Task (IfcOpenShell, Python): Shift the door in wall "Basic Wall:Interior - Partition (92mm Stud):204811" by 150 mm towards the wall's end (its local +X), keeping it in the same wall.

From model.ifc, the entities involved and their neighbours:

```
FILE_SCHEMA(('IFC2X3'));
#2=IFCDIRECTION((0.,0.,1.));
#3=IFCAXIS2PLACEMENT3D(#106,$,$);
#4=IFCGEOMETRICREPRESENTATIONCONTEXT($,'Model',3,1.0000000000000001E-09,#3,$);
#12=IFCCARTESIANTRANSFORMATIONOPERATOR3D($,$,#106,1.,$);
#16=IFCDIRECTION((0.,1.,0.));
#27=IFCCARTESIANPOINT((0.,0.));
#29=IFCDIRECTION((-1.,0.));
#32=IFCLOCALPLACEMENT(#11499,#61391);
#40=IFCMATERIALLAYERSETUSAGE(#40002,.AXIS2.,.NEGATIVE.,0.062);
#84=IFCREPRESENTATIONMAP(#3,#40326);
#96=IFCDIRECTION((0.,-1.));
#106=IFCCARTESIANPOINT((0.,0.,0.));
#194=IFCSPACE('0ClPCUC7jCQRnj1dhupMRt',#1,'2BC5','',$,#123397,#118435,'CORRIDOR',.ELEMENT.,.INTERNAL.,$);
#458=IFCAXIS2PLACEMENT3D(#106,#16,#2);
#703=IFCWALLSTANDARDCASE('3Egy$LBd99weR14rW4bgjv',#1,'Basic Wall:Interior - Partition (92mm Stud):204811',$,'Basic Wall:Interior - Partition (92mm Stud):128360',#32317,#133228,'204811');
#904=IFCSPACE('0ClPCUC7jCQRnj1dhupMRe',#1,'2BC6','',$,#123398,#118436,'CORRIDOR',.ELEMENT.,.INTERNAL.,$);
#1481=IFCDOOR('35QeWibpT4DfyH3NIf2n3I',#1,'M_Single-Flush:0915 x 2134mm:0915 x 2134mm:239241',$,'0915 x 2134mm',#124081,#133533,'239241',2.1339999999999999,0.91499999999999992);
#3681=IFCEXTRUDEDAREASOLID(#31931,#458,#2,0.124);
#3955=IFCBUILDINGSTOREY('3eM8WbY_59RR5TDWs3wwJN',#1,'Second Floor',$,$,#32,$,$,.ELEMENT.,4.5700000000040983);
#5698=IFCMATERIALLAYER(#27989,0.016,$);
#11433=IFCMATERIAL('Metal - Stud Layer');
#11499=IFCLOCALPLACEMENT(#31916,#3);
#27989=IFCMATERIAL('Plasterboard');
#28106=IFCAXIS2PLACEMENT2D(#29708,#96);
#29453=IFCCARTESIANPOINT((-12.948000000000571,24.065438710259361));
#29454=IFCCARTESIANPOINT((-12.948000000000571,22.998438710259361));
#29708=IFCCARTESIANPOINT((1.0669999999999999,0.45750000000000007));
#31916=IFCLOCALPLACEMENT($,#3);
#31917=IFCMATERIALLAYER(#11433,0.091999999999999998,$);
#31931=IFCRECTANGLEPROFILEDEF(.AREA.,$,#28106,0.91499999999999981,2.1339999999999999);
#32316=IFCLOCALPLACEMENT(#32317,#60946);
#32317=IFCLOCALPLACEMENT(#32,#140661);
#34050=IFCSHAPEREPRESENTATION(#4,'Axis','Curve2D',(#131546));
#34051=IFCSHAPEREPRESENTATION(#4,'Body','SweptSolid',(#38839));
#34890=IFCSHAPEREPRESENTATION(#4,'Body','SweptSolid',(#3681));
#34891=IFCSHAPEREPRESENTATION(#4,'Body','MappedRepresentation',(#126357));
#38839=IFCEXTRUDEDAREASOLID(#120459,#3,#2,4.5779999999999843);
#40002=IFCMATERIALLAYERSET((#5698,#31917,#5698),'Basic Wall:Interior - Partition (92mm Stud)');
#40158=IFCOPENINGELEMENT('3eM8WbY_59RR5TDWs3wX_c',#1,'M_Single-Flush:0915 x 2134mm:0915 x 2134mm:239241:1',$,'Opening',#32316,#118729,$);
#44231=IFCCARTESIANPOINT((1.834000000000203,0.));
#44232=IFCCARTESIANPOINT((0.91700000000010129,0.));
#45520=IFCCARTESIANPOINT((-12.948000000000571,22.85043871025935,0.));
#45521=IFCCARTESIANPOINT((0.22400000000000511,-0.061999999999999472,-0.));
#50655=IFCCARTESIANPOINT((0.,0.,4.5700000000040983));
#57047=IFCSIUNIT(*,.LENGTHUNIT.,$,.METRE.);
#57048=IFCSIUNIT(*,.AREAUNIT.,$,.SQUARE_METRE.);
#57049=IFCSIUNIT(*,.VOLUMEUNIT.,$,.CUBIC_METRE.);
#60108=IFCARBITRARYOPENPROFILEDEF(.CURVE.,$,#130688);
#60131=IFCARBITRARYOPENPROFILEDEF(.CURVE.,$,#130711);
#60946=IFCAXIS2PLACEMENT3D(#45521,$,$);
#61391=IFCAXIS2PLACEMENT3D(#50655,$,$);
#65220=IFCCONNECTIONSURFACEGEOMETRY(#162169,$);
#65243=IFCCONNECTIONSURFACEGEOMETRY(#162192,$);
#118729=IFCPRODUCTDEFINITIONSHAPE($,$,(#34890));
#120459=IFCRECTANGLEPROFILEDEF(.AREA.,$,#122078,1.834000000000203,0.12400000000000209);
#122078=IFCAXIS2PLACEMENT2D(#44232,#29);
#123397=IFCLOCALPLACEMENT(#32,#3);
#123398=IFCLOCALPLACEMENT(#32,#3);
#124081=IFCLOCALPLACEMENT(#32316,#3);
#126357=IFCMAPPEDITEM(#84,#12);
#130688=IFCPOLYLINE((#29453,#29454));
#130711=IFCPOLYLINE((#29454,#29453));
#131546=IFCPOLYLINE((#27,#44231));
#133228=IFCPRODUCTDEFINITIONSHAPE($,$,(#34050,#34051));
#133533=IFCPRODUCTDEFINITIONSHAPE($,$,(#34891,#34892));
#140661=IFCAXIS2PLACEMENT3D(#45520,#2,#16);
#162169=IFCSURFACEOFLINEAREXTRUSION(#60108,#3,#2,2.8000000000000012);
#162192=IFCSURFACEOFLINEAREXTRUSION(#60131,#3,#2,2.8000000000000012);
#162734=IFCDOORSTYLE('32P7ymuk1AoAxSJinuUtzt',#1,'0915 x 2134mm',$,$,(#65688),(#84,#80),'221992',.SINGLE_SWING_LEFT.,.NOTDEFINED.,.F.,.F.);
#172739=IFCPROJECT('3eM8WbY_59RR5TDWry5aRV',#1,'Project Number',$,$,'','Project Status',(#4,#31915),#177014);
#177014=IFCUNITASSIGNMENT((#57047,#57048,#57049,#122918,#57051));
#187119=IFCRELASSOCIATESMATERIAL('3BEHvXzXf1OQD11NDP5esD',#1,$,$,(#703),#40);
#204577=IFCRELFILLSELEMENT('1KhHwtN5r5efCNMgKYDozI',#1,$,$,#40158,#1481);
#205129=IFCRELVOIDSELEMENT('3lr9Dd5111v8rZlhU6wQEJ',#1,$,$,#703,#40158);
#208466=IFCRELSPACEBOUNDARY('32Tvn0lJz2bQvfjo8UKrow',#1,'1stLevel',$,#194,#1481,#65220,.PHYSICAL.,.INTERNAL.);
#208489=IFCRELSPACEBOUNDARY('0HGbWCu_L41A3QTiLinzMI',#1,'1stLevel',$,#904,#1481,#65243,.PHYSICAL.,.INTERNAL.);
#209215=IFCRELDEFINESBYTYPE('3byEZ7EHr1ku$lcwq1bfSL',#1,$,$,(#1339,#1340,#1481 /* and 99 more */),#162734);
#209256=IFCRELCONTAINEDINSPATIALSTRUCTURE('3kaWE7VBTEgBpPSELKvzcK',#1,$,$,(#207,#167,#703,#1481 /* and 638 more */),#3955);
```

```python
import numpy as np
import ifcopenshell
import ifcopenshell.api.geometry
import ifcopenshell.util.placement

model = ifcopenshell.open("model.ifc")

door = model.by_guid("35QeWibpT4DfyH3NIf2n3I")
opening = door.FillsVoids[0].RelatingOpeningElement
wall = opening.VoidsElements[0].RelatingBuildingElement

wall_matrix = ifcopenshell.util.placement.get_local_placement(wall.ObjectPlacement)
shift = wall_matrix[:3, 0] * 0.15
before = ifcopenshell.util.placement.get_local_placement(door.ObjectPlacement)[:3, 3].copy()

# The door is placed relative to its opening, so it follows when the opening moves.
matrix = ifcopenshell.util.placement.get_local_placement(opening.ObjectPlacement)
matrix[:3, 3] += shift
ifcopenshell.api.geometry.edit_object_placement(
    model, product=opening, matrix=matrix, is_si=False, should_transform_children=True
)

# Space boundary surfaces are stored in each space's coordinates; move them too.
for rel in door.ProvidesBoundaries:
    if not rel.ConnectionGeometry:
        continue
    surface = rel.ConnectionGeometry.SurfaceOnRelatingElement
    space_matrix = ifcopenshell.util.placement.get_local_placement(rel.RelatingSpace.ObjectPlacement)
    point = np.array(surface.Position.Location.Coordinates) + space_matrix[:3, :3].T @ shift
    surface.Position = model.createIfcAxis2Placement3D(
        model.createIfcCartesianPoint(point.tolist()), surface.Position.Axis, surface.Position.RefDirection
    )

after = ifcopenshell.util.placement.get_local_placement(door.ObjectPlacement)[:3, 3]
print("door moved by", (after - before).round(3) + 0.0)

model.write("model_edited.ifc")
```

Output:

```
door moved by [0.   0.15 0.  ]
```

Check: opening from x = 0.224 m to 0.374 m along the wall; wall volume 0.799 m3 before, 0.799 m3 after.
